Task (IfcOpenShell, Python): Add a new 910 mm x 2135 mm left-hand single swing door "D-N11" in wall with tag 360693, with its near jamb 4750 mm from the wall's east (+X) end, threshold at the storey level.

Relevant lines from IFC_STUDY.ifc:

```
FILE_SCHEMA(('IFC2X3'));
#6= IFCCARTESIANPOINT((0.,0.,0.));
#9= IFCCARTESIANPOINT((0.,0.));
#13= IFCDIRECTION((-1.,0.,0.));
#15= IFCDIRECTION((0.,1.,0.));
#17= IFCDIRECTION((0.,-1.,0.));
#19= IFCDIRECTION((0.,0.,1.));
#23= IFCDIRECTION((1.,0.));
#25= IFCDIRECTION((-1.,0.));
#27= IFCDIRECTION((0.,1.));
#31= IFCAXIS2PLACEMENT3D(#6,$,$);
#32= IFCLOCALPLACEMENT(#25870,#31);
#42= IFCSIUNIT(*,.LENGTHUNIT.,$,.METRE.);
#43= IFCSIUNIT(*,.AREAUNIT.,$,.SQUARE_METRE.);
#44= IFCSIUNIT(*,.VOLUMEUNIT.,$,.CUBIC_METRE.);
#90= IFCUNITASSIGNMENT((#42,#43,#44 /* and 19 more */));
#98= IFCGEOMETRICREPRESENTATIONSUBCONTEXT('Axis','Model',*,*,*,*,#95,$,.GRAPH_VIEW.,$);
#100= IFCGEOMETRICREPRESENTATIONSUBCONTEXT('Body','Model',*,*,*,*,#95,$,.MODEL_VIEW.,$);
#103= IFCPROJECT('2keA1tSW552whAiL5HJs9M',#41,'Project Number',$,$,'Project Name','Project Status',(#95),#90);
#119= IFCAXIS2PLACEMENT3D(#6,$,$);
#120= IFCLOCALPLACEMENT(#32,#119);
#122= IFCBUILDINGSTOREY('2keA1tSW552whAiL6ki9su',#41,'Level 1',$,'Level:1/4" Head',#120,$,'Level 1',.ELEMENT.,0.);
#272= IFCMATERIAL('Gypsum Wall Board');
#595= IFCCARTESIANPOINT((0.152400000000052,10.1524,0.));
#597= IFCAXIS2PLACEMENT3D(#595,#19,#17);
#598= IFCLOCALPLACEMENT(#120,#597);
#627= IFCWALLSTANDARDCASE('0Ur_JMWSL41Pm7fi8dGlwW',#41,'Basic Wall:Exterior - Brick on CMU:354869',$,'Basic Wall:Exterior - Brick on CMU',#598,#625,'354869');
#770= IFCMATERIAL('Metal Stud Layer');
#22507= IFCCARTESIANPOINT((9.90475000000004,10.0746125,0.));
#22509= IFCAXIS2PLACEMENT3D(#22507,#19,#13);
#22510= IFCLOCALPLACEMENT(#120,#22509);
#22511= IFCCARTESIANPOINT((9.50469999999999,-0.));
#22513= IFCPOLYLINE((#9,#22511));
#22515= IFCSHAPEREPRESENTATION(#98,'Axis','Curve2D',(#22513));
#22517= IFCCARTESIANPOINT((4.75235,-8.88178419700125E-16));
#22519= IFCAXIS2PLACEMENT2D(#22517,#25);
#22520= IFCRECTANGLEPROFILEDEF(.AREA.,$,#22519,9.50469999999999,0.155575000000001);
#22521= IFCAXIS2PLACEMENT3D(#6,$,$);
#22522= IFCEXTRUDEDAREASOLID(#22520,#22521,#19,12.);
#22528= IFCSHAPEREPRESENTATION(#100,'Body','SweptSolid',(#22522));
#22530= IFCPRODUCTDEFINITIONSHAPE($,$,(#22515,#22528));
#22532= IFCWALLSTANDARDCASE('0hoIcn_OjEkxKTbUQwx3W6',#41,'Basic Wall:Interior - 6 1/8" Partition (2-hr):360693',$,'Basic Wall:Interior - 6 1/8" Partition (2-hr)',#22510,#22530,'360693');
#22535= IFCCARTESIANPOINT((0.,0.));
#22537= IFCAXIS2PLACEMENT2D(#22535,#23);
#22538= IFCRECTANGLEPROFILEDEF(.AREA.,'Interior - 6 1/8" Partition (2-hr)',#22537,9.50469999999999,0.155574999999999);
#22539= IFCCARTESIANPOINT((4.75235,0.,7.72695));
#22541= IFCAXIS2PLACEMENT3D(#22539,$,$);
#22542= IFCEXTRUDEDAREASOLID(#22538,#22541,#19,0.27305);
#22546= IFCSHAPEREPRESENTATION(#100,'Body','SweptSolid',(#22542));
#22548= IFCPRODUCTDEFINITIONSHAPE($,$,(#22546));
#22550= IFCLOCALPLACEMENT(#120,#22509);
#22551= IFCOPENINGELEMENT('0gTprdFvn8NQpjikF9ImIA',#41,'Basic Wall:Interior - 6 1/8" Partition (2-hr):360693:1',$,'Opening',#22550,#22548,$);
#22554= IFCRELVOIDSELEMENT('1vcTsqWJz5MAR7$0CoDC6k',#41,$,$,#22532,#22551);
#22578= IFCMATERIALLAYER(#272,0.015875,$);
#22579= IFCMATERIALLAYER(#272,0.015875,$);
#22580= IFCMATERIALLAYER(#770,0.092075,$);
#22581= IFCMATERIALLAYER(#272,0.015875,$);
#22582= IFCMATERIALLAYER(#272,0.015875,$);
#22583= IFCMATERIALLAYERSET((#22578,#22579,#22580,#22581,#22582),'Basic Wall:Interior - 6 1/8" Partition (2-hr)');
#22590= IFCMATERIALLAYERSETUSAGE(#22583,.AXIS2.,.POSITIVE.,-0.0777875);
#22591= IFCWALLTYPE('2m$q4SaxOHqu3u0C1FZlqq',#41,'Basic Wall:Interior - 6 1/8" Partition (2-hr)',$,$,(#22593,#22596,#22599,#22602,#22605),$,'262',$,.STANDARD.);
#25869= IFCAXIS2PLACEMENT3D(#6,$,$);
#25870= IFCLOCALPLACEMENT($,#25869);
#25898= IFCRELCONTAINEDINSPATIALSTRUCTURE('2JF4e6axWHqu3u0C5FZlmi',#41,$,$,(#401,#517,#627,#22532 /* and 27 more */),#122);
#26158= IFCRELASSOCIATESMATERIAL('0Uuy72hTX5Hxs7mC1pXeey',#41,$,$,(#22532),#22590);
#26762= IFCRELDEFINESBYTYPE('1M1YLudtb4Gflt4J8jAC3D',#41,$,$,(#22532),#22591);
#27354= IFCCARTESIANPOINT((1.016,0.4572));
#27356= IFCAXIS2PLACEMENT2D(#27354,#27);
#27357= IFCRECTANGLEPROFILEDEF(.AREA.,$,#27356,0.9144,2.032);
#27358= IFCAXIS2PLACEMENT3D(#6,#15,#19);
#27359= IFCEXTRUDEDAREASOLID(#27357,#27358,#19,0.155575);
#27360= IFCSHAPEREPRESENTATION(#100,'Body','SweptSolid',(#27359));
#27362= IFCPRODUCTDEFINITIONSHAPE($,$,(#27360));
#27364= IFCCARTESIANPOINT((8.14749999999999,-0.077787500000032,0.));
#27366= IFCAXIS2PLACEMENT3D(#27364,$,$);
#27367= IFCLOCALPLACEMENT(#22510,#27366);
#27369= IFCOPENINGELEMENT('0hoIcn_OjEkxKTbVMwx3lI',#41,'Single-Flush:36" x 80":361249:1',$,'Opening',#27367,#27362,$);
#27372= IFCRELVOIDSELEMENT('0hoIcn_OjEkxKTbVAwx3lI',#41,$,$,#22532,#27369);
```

```python
import numpy as np
import ifcopenshell
import ifcopenshell.api.feature
import ifcopenshell.api.geometry
import ifcopenshell.api.root
import ifcopenshell.api.spatial
import ifcopenshell.api.type
import ifcopenshell.geom
import ifcopenshell.util.element
import ifcopenshell.util.placement
import ifcopenshell.util.representation
import ifcopenshell.util.shape
import ifcopenshell.util.unit

model = ifcopenshell.open("IFC_STUDY.ifc")
unit_scale = ifcopenshell.util.unit.calculate_unit_scale(model)
settings = ifcopenshell.geom.settings()


def volume(element):
    """Net volume in cubic metres, openings subtracted."""
    shape = ifcopenshell.geom.create_shape(settings, element)
    return ifcopenshell.util.shape.get_volume(shape.geometry)


wall = model.by_id(22532)
storey = ifcopenshell.util.element.get_container(wall, ifc_class="IfcBuildingStorey")
context = ifcopenshell.util.representation.get_context(model, "Model", "Body", "MODEL_VIEW")
before = volume(wall)

width, height, from_end, sill = 0.91, 2.135, 4.75, 0.0  # metres

# The wall runs along its own X axis, and the end named is its -X end.
wall_shape = ifcopenshell.geom.create_shape(settings, wall)
x, y, z = ifcopenshell.util.shape.get_vertices(wall_shape.geometry).T
start = x.min() + from_end
face, thickness = float(y.min()), float(y.max() - y.min())
wall_matrix = ifcopenshell.util.placement.get_local_placement(wall.ObjectPlacement)
level = ifcopenshell.util.placement.get_local_placement(storey.ObjectPlacement)[2, 3]


def in_wall(x, y):
    """Placement at x, y metres in the wall's axes, at sill height."""
    matrix = wall_matrix.copy()
    matrix[:, 3] = wall_matrix @ np.array([x / unit_scale, y / unit_scale, 0.0, 1.0])
    matrix[2, 3] = level + sill / unit_scale
    return matrix


# Opening: a box that overshoots both wall faces by 50 mm.
opening = ifcopenshell.api.root.create_entity(model, ifc_class="IfcOpeningElement")
box = ifcopenshell.api.geometry.add_wall_representation(
    model, context=context, length=width, height=height, thickness=thickness + 0.1
)
ifcopenshell.api.geometry.assign_representation(model, product=opening, representation=box)
ifcopenshell.api.geometry.edit_object_placement(model, product=opening, matrix=in_wall(start, face - 0.05), is_si=False)
ifcopenshell.api.feature.add_feature(model, feature=opening, element=wall)

door = ifcopenshell.api.root.create_entity(model, ifc_class="IfcDoor", name="D-N11")
door.OverallWidth, door.OverallHeight = width / unit_scale, height / unit_scale
body = ifcopenshell.api.geometry.add_door_representation(
    model,
    context=context,
    overall_width=door.OverallWidth,
    overall_height=door.OverallHeight,
    operation_type="SINGLE_SWING_LEFT",
    lining_properties={"LiningDepth": thickness / unit_scale, "ThresholdDepth": thickness / unit_scale},
)
ifcopenshell.api.geometry.assign_representation(model, product=door, representation=body)
ifcopenshell.api.spatial.assign_container(model, products=[door], relating_structure=storey)
fills = ifcopenshell.api.feature.add_filling(model, opening=opening, element=door)
fills.OwnerHistory = door.OwnerHistory  # required in IFC2X3

# IFC2X3 keeps the operation on the door style.
style = ifcopenshell.api.root.create_entity(model, ifc_class="IfcDoorStyle", name="D-N11")
style.OperationType, style.ConstructionType = "SINGLE_SWING_LEFT", "NOTDEFINED"
style.ParameterTakesPrecedence = style.Sizeable = False
ifcopenshell.api.type.assign_type(model, related_objects=[door], relating_type=style)

# The lining spans the wall, so the door starts at the wall face.
ifcopenshell.api.geometry.edit_object_placement(model, product=door, matrix=in_wall(start, face), is_si=False)

after = volume(wall)

print(f"wall volume {before:.3f} -> {after:.3f} m3")

model.write("IFC_STUDY_v2.ifc")
```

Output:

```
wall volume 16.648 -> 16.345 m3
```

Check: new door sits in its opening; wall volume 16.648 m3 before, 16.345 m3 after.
